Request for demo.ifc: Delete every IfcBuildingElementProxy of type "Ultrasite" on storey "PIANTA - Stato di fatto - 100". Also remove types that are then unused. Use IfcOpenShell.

First a look at what the model holds.

```python
import ifcopenshell
import ifcopenshell.util.element

model = ifcopenshell.open("demo.ifc")
print(model.schema)
storey = next(s for s in model.by_type("IfcBuildingStorey") if s.Name == "PIANTA - Stato di fatto - 100")
proxies = [e for e in ifcopenshell.util.element.get_decomposition(storey) if e.is_a("IfcBuildingElementProxy")]
seen = {}
for e in proxies:
    element_type = ifcopenshell.util.element.get_type(e)
    name = element_type.Name if element_type not in (None, e) else None
    seen[name] = seen.get(name, 0) + 1
for name, count in sorted(seen.items(), key=str):
    print(count, "x", name)
```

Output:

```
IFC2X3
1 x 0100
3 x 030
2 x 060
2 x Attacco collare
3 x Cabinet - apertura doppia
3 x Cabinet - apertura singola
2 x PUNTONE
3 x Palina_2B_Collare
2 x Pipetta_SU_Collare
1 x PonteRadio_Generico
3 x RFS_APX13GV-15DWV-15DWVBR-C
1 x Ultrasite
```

```python
import ifcopenshell
import ifcopenshell.api.root
import ifcopenshell.util.element

model = ifcopenshell.open("demo.ifc")

storey = next(s for s in model.by_type("IfcBuildingStorey") if s.Name == "PIANTA - Stato di fatto - 100")
proxies = [e for e in ifcopenshell.util.element.get_decomposition(storey) if e.is_a("IfcBuildingElementProxy")]
targets = [e for e in proxies if (t := ifcopenshell.util.element.get_type(e)) not in (None, e) and t.Name == "Ultrasite"]
types = {ifcopenshell.util.element.get_type(e) for e in targets} - {None, *targets}

for e in targets:
    ifcopenshell.api.root.remove_product(model, product=e)
print(len(targets), "removed")

unused = [t for t in types if not ifcopenshell.util.element.get_types(t)]
for t in unused:
    ifcopenshell.api.root.remove_product(model, product=t)
print(len(unused), "unused types removed")

model.write("demo_rev.ifc")
```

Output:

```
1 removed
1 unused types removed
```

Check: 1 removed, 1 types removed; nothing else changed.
